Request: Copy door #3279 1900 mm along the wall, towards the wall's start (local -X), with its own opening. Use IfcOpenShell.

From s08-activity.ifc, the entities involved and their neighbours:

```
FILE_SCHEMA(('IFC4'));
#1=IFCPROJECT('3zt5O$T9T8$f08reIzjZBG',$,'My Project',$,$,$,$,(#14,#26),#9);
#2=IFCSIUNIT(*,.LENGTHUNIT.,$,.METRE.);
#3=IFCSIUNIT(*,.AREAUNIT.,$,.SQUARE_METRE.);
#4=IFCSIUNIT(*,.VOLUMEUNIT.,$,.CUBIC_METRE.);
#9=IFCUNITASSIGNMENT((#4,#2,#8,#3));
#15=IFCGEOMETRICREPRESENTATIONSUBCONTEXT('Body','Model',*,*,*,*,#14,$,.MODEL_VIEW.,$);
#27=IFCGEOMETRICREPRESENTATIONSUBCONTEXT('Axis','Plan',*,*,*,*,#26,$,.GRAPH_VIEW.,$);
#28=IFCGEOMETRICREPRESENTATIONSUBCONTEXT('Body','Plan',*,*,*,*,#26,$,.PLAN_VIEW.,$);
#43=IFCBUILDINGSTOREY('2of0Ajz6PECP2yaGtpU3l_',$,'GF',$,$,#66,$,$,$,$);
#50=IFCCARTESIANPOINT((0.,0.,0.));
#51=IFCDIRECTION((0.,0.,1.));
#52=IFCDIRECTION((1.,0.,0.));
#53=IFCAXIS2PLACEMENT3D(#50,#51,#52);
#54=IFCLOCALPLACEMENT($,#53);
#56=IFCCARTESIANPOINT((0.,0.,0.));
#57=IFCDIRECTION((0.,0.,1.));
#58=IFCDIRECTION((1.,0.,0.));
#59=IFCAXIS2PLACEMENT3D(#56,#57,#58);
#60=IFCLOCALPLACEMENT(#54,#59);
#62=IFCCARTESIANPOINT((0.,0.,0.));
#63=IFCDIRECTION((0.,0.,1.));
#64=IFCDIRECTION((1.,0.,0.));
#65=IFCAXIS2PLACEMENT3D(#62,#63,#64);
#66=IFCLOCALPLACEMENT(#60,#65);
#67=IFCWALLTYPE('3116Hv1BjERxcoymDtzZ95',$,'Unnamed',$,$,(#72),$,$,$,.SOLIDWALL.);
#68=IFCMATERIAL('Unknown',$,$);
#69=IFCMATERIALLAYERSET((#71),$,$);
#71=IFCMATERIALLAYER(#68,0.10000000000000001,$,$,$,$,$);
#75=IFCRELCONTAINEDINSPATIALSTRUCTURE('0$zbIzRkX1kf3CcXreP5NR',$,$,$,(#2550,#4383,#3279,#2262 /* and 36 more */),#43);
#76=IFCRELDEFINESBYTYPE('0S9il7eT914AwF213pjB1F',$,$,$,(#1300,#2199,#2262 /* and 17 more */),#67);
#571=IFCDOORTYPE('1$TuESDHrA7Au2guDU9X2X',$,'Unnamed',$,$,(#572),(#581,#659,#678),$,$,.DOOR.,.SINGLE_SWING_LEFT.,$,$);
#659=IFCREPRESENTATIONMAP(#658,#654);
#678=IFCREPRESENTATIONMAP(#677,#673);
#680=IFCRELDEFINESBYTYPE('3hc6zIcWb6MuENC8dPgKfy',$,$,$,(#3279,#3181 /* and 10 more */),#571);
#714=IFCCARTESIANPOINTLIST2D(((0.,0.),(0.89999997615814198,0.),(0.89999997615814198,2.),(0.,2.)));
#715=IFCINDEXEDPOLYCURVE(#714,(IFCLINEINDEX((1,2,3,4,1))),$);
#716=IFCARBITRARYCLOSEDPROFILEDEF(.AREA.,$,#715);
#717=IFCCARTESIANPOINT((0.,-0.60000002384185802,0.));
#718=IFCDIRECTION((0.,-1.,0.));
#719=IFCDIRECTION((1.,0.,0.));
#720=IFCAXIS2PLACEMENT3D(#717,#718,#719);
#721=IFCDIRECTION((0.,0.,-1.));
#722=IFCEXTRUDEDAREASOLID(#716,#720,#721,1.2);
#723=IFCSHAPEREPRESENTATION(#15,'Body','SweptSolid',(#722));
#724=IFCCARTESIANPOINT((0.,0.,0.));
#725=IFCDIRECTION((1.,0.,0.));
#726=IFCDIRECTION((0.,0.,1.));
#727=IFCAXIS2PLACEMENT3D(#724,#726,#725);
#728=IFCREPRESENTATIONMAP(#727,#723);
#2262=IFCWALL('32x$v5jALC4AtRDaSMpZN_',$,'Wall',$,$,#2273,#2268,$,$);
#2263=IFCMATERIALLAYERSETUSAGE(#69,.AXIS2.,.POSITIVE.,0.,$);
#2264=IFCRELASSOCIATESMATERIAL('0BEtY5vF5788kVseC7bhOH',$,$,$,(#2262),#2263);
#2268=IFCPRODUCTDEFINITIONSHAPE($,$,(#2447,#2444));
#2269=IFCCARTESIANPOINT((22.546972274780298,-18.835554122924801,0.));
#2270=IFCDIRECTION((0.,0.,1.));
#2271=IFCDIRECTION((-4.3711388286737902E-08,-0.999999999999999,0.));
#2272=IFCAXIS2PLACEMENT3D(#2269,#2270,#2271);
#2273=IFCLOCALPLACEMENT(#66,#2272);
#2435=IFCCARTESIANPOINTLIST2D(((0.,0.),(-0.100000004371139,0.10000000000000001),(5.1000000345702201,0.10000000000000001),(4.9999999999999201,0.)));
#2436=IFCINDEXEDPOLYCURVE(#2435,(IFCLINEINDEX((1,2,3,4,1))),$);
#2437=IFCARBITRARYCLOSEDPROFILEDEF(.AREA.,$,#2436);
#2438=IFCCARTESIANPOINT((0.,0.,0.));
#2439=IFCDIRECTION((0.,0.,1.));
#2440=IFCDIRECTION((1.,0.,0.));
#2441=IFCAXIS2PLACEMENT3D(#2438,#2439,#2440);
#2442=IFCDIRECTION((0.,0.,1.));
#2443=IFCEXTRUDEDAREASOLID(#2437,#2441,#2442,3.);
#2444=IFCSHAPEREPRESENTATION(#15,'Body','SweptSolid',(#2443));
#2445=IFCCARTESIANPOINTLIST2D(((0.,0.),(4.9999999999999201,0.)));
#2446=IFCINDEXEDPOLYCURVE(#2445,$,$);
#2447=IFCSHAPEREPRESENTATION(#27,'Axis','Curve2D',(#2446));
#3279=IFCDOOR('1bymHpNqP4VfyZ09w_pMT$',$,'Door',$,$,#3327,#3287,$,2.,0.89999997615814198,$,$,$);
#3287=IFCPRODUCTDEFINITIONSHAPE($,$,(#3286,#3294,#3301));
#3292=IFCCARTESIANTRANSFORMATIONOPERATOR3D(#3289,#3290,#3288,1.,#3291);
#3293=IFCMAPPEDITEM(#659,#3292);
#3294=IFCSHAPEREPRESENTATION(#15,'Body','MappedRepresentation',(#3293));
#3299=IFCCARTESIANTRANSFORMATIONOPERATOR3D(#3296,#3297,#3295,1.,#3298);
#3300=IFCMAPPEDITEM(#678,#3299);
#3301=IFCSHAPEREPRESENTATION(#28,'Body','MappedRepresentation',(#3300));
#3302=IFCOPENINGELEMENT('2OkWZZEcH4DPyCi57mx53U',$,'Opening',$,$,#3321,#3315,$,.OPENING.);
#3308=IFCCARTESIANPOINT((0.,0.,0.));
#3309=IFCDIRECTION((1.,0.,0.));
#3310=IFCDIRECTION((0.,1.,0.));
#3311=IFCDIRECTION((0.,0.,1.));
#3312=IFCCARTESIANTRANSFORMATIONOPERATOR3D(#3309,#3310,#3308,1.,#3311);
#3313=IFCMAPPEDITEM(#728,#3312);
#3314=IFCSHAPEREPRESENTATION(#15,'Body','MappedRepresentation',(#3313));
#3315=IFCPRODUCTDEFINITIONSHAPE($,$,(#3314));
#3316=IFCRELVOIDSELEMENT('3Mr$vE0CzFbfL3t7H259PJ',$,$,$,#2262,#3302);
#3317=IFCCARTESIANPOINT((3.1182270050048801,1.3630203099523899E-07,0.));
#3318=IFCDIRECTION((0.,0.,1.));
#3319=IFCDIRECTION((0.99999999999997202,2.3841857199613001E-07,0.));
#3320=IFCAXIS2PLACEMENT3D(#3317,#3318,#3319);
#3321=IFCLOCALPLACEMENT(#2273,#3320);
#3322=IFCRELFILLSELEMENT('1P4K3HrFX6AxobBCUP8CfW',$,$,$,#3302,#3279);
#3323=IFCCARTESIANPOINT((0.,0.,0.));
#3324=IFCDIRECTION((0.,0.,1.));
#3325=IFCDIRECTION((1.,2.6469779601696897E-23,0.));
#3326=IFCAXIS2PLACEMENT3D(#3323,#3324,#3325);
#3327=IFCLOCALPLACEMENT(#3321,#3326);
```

```python
import ifcopenshell
import ifcopenshell.api.feature
import ifcopenshell.api.geometry
import ifcopenshell.api.root
import ifcopenshell.geom
import ifcopenshell.util.element
import ifcopenshell.util.placement
import ifcopenshell.util.shape
import ifcopenshell.util.unit

model = ifcopenshell.open("s08-activity.ifc")
unit_scale = ifcopenshell.util.unit.calculate_unit_scale(model)
settings = ifcopenshell.geom.settings()


def volume(element):
    """Net volume in cubic metres, openings subtracted."""
    shape = ifcopenshell.geom.create_shape(settings, element)
    return ifcopenshell.util.shape.get_volume(shape.geometry)


door = model.by_guid("1bymHpNqP4VfyZ09w_pMT$")
opening = door.FillsVoids[0].RelatingOpeningElement
wall = opening.VoidsElements[0].RelatingBuildingElement
before = volume(wall)
shift = ifcopenshell.util.placement.get_local_placement(wall.ObjectPlacement)[:3, 0] * -1.9 / unit_scale

# copy_class copies the void relationship, type, container and properties, but no geometry.
new_opening = ifcopenshell.api.root.copy_class(model, product=opening)
new_opening.Representation = ifcopenshell.util.element.copy_deep(
    model, opening.Representation, exclude=["IfcGeometricRepresentationContext", "IfcRepresentationMap"]
)
new_door = ifcopenshell.api.root.copy_class(model, product=door)
new_door.Representation = ifcopenshell.util.element.copy_deep(
    model, door.Representation, exclude=["IfcGeometricRepresentationContext", "IfcRepresentationMap"]
)
ifcopenshell.api.feature.add_filling(model, opening=new_opening, element=new_door)

for old, new in ((opening, new_opening), (door, new_door)):
    matrix = ifcopenshell.util.placement.get_local_placement(old.ObjectPlacement)
    matrix[:3, 3] += shift
    ifcopenshell.api.geometry.edit_object_placement(model, product=new, matrix=matrix, is_si=False)

after = volume(wall)

print(f"wall volume {before:.3f} -> {after:.3f} m3")

model.write("s08-activity_edited.ifc")
```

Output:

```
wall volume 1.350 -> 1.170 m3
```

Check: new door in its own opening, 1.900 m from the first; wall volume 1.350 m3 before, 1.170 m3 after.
